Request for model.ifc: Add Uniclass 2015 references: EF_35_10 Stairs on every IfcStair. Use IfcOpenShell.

First a look at what the model holds.

```python
import ifcopenshell

model = ifcopenshell.open("model.ifc")
print(model.schema)
print("classifications:", [c.Name for c in model.by_type("IfcClassification")])
for ifc_class in ("IfcDoor", "IfcRoof", "IfcStair", "IfcWall", "IfcWindow"):
    print(ifc_class, len(model.by_type(ifc_class)))
```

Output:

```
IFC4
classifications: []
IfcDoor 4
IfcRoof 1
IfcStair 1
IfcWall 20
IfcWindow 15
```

```python
import ifcopenshell
import ifcopenshell.api.classification

model = ifcopenshell.open("model.ifc")

system = ifcopenshell.api.classification.add_classification(model, classification="Uniclass 2015")

codes = {
    "IfcStair": ("EF_35_10", "Stairs"),
}
for ifc_class, (code, name) in codes.items():
    products = model.by_type(ifc_class)
    ifcopenshell.api.classification.add_reference(
        model, products=products, classification=system, identification=code, name=name
    )
    print(code, len(products))

model.write("model_edited.ifc")
```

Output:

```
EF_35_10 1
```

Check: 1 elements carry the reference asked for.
